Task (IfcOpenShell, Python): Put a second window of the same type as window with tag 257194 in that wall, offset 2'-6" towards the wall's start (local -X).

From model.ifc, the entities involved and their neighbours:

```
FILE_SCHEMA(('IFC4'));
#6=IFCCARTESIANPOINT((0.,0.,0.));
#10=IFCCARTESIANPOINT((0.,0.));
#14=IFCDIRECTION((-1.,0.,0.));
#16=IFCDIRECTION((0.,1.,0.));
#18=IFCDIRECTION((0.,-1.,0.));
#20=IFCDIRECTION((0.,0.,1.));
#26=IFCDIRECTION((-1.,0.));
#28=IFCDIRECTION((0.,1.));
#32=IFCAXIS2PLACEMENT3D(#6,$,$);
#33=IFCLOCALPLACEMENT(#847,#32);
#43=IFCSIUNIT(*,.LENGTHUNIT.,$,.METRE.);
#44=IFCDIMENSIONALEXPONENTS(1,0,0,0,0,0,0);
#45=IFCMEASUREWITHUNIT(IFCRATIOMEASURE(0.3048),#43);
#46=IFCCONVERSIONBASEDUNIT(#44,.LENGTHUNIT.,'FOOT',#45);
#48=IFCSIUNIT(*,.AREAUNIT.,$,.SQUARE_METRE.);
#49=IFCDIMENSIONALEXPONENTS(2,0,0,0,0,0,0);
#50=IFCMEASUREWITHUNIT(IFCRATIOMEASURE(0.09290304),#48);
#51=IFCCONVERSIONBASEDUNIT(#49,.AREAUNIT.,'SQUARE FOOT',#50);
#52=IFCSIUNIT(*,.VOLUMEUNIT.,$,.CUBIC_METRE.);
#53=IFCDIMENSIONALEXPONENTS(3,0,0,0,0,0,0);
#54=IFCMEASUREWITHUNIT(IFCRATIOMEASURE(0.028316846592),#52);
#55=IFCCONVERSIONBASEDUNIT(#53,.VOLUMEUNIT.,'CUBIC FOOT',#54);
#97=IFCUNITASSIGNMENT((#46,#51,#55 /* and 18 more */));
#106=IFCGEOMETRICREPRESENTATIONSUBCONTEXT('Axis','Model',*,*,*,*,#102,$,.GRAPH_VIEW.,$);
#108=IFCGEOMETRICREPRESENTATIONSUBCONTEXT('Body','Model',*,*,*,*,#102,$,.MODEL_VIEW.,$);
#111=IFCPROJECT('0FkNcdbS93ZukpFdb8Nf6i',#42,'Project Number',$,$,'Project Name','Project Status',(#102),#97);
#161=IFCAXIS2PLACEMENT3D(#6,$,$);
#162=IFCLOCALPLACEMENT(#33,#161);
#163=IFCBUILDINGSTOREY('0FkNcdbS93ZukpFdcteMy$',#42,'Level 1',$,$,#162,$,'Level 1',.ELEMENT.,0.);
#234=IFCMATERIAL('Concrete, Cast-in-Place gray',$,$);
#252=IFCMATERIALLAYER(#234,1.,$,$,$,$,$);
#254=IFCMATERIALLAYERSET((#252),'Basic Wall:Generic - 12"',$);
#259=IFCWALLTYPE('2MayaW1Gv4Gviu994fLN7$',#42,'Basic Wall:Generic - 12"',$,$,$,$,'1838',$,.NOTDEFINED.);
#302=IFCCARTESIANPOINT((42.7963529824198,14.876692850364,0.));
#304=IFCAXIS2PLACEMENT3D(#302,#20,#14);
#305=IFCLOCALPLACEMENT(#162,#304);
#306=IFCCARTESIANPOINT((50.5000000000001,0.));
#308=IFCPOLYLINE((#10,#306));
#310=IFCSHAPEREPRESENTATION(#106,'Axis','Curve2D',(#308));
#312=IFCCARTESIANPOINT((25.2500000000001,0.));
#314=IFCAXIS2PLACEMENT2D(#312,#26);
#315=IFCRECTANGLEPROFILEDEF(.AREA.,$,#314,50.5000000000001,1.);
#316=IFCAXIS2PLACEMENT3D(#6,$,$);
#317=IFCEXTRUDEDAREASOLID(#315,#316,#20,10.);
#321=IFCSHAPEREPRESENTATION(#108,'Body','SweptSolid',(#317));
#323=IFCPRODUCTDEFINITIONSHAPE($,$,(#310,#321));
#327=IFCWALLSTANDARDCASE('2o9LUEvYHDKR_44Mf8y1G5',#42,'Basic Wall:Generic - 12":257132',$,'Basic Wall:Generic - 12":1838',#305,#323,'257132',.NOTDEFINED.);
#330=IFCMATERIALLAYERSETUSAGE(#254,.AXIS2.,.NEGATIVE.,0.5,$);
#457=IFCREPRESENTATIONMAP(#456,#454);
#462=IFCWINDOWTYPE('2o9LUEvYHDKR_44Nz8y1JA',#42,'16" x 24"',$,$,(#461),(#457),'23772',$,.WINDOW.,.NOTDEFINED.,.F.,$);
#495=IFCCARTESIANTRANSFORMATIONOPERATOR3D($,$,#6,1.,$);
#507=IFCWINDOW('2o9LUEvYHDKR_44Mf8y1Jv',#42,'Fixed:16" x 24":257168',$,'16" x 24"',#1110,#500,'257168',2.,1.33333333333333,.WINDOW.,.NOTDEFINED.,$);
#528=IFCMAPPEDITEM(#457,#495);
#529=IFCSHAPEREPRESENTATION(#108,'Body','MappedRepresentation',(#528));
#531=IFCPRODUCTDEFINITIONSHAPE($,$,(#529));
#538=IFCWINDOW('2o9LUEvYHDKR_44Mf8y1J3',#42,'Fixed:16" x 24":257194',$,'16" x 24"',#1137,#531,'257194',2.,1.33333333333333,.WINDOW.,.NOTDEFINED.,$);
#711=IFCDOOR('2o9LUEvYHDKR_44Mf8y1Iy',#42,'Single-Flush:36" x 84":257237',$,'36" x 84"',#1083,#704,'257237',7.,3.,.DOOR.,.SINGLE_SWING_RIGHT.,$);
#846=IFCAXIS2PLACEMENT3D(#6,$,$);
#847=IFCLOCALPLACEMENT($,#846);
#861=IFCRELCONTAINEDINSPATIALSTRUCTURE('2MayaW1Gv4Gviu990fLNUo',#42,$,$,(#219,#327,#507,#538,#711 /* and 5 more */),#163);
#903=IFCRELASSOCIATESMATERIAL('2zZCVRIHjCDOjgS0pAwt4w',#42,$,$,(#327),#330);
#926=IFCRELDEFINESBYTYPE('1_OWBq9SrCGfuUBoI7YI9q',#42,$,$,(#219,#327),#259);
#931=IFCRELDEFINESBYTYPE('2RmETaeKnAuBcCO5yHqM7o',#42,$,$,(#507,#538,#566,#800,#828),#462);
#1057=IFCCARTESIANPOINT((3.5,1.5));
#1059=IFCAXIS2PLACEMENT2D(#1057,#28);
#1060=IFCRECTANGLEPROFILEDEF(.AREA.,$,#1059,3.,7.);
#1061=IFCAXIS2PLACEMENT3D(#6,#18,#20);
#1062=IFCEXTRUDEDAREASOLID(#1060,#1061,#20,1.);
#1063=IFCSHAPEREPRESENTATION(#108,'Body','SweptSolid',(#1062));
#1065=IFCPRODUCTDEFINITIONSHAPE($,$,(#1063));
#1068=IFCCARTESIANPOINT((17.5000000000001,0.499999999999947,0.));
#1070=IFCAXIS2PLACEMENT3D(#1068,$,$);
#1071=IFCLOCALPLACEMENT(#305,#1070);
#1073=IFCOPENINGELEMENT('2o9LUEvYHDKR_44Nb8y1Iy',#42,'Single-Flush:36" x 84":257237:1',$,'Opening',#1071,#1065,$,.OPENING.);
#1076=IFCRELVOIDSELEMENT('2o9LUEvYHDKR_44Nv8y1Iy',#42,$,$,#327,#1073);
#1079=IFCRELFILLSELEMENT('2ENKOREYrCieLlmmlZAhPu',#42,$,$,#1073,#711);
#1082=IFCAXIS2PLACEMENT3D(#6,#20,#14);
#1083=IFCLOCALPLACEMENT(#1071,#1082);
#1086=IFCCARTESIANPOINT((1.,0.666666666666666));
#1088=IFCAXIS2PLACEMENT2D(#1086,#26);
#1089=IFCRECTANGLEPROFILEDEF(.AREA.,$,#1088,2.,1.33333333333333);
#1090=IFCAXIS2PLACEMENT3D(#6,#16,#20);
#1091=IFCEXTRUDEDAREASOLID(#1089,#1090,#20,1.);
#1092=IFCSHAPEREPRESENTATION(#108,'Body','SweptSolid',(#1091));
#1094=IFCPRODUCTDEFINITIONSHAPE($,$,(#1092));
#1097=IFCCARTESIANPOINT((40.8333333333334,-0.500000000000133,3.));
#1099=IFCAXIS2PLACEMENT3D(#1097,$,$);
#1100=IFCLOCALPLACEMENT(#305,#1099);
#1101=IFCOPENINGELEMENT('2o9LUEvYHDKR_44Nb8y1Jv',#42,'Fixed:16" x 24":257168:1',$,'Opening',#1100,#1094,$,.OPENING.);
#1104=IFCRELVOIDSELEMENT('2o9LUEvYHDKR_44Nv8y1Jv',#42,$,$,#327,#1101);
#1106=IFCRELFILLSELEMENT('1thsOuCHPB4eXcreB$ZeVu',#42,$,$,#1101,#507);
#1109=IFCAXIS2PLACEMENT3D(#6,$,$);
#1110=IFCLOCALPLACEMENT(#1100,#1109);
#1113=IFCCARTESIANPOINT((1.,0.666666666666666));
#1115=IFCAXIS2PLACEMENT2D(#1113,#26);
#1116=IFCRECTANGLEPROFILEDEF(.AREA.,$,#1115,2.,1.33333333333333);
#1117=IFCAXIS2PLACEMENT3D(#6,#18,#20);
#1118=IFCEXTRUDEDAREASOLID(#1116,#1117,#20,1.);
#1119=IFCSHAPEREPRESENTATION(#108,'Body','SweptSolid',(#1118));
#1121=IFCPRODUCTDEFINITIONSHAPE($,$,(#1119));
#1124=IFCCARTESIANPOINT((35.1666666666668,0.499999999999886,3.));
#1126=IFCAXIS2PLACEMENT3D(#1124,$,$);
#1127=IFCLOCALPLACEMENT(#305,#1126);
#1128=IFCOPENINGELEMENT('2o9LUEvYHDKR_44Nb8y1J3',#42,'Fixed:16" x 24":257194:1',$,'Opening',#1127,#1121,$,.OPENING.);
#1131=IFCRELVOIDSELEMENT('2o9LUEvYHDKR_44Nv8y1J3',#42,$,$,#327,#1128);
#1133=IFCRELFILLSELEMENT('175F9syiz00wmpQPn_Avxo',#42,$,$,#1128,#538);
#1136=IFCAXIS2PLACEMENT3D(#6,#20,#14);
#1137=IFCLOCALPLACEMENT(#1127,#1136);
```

```python
import ifcopenshell
import ifcopenshell.api.feature
import ifcopenshell.api.geometry
import ifcopenshell.api.root
import ifcopenshell.geom
import ifcopenshell.util.element
import ifcopenshell.util.placement
import ifcopenshell.util.shape
import ifcopenshell.util.unit

model = ifcopenshell.open("model.ifc")
unit_scale = ifcopenshell.util.unit.calculate_unit_scale(model)
settings = ifcopenshell.geom.settings()


def volume(element):
    """Net volume in cubic metres, openings subtracted."""
    shape = ifcopenshell.geom.create_shape(settings, element)
    return ifcopenshell.util.shape.get_volume(shape.geometry)


def reuse_history(source, copy):
    """copy_class also copies each property set's owner history, people and application; keep the originals."""
    for rel in copy.IsDefinedBy:
        if rel.is_a("IfcRelDefinesByProperties") and (history := rel.RelatingPropertyDefinition.OwnerHistory):
            rel.RelatingPropertyDefinition.OwnerHistory = source.OwnerHistory
            ifcopenshell.util.element.remove_deep2(model, history)


window = model.by_guid("2o9LUEvYHDKR_44Mf8y1J3")
opening = window.FillsVoids[0].RelatingOpeningElement
wall = opening.VoidsElements[0].RelatingBuildingElement
before = volume(wall)
shift = ifcopenshell.util.placement.get_local_placement(wall.ObjectPlacement)[:3, 0] * -30 * 0.0254 / unit_scale

# copy_class copies the void relationship, type, container and properties, but no geometry.
new_opening = ifcopenshell.api.root.copy_class(model, product=opening)
new_opening.Representation = ifcopenshell.util.element.copy_deep(
    model, opening.Representation, exclude=["IfcGeometricRepresentationContext", "IfcRepresentationMap"]
)
new_opening.Name = 'Fixed:16" x 24"'
new_window = ifcopenshell.api.root.copy_class(model, product=window)
new_window.Representation = ifcopenshell.util.element.copy_deep(
    model, window.Representation, exclude=["IfcGeometricRepresentationContext", "IfcRepresentationMap"]
)
new_window.Name = 'Fixed:16" x 24"'
new_window.Tag = None
reuse_history(window, new_window)
ifcopenshell.api.feature.add_filling(model, opening=new_opening, element=new_window)

for old, new in ((opening, new_opening), (window, new_window)):
    matrix = ifcopenshell.util.placement.get_local_placement(old.ObjectPlacement)
    matrix[:3, 3] += shift
    ifcopenshell.api.geometry.edit_object_placement(model, product=new, matrix=matrix, is_si=False)

after = volume(wall)

print(f"wall volume {before:.3f} -> {after:.3f} m3")

model.write("model_edited.ifc")
```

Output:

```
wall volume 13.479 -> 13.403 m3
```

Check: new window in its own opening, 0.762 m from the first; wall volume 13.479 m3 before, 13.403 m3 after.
